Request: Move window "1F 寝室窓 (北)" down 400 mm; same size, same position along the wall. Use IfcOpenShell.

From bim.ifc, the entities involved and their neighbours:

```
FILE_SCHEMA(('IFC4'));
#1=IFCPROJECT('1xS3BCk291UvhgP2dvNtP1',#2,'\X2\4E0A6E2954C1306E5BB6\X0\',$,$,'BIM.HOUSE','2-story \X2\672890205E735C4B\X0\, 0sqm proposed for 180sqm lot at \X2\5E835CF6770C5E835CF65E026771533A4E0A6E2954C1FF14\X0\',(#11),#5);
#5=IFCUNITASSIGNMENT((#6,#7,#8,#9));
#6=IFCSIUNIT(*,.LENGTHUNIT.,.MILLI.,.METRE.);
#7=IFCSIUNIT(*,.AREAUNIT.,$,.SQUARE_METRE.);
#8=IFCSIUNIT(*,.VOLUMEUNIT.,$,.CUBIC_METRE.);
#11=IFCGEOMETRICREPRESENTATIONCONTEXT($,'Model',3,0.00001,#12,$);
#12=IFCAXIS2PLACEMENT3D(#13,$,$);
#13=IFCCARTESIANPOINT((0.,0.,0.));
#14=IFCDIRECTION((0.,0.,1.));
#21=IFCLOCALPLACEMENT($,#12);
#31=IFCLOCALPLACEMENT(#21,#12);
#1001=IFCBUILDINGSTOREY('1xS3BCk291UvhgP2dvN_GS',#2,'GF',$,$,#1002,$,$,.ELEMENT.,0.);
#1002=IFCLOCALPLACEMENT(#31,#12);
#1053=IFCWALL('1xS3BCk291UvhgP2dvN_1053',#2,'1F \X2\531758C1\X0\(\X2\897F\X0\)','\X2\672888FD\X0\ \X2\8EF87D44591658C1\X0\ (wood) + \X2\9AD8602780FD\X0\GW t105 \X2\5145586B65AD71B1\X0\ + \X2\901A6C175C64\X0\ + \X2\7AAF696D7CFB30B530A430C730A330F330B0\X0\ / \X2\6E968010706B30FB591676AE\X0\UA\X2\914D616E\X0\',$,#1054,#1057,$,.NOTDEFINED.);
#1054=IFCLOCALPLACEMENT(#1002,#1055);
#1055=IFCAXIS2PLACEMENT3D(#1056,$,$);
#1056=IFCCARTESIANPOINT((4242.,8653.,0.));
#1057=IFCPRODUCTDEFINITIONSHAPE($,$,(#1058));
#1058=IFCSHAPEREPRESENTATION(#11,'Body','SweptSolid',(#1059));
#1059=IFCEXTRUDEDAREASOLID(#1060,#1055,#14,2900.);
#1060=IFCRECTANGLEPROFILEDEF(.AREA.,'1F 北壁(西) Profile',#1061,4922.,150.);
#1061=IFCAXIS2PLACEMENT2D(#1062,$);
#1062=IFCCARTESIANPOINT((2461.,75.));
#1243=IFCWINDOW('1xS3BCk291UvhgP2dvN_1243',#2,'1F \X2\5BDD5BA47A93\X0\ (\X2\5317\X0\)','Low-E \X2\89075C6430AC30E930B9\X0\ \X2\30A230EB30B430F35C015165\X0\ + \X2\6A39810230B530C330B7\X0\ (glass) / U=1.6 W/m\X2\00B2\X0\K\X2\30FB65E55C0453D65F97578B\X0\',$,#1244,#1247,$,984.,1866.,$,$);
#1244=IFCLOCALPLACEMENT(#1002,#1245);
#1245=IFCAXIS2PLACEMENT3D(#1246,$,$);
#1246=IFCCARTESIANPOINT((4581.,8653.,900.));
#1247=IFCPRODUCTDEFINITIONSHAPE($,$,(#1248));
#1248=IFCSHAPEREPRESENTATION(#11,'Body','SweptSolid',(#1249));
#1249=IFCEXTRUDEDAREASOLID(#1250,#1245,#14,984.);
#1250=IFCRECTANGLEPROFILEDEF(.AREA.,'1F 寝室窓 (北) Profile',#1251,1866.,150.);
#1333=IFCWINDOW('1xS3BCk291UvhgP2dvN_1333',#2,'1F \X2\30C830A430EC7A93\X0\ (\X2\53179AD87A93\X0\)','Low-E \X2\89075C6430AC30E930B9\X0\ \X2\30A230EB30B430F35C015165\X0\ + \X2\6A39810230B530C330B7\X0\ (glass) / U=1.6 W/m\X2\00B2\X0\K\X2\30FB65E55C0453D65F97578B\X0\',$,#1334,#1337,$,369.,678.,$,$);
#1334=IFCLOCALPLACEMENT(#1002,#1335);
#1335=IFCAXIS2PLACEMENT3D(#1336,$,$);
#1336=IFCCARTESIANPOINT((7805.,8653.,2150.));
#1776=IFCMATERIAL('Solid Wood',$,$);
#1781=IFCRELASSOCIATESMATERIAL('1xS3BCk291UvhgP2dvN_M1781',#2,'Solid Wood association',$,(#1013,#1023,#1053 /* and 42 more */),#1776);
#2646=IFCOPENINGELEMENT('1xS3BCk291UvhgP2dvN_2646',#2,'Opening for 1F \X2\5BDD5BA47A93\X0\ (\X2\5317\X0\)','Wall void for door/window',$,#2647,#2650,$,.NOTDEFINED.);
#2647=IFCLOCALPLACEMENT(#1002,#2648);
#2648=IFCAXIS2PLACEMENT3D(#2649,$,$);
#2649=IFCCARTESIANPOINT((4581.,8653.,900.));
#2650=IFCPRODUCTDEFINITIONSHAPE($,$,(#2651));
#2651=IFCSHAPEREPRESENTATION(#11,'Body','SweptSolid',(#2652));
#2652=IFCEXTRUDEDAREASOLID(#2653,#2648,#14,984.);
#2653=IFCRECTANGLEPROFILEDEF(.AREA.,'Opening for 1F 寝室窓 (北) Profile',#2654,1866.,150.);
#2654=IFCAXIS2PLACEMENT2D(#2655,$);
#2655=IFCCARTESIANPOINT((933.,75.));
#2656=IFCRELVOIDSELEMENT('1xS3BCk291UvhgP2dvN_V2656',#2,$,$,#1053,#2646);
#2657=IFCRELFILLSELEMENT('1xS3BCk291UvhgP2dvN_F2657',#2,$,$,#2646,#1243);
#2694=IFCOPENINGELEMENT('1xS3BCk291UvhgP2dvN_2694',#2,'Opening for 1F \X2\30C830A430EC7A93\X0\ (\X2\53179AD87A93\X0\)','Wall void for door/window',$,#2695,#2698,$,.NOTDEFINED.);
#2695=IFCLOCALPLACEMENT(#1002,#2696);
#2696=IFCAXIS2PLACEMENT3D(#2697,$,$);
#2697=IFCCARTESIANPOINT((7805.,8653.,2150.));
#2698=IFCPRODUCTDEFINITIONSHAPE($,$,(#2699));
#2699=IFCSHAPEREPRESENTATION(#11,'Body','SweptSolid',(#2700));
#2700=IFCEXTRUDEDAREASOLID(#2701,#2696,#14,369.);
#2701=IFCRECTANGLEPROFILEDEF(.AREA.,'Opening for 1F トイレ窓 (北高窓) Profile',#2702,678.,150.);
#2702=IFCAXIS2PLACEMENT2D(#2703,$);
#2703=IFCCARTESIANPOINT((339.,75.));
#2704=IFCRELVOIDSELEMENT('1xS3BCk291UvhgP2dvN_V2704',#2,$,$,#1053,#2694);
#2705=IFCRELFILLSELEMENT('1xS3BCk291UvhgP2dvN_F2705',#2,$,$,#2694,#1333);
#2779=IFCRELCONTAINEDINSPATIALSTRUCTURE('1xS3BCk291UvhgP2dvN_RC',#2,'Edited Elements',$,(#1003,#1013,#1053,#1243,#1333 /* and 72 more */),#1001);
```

```python
import numpy as np
import ifcopenshell
import ifcopenshell.api.geometry
import ifcopenshell.util.placement
import ifcopenshell.util.unit

model = ifcopenshell.open("bim.ifc")
unit_scale = ifcopenshell.util.unit.calculate_unit_scale(model)

window = model.by_guid("1xS3BCk291UvhgP2dvN_1243")
opening = window.FillsVoids[0].RelatingOpeningElement
dz = -400.0

shift = np.array([0.0, 0.0, dz])
# The window is not placed relative to its opening, so move both.
for product in (opening, window):
    matrix = ifcopenshell.util.placement.get_local_placement(product.ObjectPlacement)
    matrix[:3, 3] += shift
    ifcopenshell.api.geometry.edit_object_placement(model, product=product, matrix=matrix, is_si=False)

print(f"moved by {dz * unit_scale:+.3f} m")

model.write("bim_v2.ifc")
```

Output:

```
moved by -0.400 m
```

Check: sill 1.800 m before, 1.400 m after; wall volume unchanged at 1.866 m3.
